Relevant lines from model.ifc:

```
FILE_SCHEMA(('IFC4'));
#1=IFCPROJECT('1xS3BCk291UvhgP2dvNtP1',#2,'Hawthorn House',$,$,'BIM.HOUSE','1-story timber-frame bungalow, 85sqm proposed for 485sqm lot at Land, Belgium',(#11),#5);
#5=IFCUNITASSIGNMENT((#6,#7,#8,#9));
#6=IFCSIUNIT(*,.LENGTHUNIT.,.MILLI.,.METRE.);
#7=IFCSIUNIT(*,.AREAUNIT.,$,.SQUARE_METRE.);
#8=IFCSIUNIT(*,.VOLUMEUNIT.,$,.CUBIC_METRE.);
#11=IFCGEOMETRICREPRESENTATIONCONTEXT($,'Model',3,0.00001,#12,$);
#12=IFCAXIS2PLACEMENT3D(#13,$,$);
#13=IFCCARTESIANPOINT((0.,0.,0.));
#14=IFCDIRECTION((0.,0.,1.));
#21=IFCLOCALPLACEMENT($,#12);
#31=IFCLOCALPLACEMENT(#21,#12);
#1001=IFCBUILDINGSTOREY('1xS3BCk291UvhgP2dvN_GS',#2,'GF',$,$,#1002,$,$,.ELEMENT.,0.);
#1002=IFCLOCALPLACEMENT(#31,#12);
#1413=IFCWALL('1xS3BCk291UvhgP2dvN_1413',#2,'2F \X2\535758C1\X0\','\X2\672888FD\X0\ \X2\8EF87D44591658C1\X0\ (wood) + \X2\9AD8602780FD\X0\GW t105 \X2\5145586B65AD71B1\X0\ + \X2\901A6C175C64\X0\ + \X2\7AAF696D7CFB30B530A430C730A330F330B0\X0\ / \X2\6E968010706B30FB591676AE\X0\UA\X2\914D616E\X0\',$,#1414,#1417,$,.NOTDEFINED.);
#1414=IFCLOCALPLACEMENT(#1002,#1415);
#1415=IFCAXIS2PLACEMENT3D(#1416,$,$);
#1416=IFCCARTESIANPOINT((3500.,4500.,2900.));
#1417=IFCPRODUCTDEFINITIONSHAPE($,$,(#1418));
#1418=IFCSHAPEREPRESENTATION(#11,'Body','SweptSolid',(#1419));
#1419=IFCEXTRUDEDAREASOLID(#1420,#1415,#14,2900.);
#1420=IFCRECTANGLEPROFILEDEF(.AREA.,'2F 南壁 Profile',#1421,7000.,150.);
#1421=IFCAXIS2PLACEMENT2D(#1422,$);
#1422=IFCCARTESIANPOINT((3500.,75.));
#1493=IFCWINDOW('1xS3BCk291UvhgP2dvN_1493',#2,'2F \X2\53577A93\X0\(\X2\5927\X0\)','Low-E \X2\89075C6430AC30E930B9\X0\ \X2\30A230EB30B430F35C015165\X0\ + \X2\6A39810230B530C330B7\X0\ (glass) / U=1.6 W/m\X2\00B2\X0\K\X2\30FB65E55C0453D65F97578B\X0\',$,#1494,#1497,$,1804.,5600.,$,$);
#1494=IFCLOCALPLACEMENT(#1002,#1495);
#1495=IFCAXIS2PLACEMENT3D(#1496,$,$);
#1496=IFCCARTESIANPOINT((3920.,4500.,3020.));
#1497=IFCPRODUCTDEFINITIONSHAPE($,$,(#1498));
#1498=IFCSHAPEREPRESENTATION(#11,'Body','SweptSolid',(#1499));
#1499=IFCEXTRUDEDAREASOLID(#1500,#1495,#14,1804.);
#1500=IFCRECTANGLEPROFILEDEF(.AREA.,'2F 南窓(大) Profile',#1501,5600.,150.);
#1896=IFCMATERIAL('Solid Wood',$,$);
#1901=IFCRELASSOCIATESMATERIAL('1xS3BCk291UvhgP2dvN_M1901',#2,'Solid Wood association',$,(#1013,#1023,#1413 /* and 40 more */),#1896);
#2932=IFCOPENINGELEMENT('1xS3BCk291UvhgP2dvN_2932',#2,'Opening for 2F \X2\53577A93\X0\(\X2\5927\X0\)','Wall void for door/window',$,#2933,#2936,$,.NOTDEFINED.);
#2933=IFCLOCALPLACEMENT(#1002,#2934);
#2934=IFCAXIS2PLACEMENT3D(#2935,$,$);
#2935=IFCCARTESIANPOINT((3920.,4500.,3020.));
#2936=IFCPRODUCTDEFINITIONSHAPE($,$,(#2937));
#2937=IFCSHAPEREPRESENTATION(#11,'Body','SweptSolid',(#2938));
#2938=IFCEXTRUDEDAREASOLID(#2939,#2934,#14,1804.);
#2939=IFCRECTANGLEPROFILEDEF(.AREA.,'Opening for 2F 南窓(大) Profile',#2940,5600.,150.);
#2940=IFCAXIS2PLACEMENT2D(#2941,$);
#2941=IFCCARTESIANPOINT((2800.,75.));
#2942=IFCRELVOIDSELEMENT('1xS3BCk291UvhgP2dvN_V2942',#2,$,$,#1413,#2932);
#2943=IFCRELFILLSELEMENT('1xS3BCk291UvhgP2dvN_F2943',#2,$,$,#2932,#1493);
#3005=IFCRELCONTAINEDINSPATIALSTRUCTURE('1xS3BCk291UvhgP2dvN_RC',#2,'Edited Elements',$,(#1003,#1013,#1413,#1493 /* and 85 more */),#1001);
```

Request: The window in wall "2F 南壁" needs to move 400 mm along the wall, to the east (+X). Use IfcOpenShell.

```python
import ifcopenshell
import ifcopenshell.api.geometry
import ifcopenshell.util.placement

model = ifcopenshell.open("model.ifc")

window = model.by_guid("1xS3BCk291UvhgP2dvN_1493")
opening = window.FillsVoids[0].RelatingOpeningElement
wall = opening.VoidsElements[0].RelatingBuildingElement

wall_matrix = ifcopenshell.util.placement.get_local_placement(wall.ObjectPlacement)
shift = wall_matrix[:3, 0] * 400.0
before = ifcopenshell.util.placement.get_local_placement(window.ObjectPlacement)[:3, 3].copy()

# The window is not placed relative to its opening, so move both.
for product in (opening, window):
    matrix = ifcopenshell.util.placement.get_local_placement(product.ObjectPlacement)
    matrix[:3, 3] += shift
    ifcopenshell.api.geometry.edit_object_placement(model, product=product, matrix=matrix, is_si=False)

after = ifcopenshell.util.placement.get_local_placement(window.ObjectPlacement)[:3, 3]
print("window moved by", (after - before).round(3) + 0.0)

model.write("model_edited.ifc")
```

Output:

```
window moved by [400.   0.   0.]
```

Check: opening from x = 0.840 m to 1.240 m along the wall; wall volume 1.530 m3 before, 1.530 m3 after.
